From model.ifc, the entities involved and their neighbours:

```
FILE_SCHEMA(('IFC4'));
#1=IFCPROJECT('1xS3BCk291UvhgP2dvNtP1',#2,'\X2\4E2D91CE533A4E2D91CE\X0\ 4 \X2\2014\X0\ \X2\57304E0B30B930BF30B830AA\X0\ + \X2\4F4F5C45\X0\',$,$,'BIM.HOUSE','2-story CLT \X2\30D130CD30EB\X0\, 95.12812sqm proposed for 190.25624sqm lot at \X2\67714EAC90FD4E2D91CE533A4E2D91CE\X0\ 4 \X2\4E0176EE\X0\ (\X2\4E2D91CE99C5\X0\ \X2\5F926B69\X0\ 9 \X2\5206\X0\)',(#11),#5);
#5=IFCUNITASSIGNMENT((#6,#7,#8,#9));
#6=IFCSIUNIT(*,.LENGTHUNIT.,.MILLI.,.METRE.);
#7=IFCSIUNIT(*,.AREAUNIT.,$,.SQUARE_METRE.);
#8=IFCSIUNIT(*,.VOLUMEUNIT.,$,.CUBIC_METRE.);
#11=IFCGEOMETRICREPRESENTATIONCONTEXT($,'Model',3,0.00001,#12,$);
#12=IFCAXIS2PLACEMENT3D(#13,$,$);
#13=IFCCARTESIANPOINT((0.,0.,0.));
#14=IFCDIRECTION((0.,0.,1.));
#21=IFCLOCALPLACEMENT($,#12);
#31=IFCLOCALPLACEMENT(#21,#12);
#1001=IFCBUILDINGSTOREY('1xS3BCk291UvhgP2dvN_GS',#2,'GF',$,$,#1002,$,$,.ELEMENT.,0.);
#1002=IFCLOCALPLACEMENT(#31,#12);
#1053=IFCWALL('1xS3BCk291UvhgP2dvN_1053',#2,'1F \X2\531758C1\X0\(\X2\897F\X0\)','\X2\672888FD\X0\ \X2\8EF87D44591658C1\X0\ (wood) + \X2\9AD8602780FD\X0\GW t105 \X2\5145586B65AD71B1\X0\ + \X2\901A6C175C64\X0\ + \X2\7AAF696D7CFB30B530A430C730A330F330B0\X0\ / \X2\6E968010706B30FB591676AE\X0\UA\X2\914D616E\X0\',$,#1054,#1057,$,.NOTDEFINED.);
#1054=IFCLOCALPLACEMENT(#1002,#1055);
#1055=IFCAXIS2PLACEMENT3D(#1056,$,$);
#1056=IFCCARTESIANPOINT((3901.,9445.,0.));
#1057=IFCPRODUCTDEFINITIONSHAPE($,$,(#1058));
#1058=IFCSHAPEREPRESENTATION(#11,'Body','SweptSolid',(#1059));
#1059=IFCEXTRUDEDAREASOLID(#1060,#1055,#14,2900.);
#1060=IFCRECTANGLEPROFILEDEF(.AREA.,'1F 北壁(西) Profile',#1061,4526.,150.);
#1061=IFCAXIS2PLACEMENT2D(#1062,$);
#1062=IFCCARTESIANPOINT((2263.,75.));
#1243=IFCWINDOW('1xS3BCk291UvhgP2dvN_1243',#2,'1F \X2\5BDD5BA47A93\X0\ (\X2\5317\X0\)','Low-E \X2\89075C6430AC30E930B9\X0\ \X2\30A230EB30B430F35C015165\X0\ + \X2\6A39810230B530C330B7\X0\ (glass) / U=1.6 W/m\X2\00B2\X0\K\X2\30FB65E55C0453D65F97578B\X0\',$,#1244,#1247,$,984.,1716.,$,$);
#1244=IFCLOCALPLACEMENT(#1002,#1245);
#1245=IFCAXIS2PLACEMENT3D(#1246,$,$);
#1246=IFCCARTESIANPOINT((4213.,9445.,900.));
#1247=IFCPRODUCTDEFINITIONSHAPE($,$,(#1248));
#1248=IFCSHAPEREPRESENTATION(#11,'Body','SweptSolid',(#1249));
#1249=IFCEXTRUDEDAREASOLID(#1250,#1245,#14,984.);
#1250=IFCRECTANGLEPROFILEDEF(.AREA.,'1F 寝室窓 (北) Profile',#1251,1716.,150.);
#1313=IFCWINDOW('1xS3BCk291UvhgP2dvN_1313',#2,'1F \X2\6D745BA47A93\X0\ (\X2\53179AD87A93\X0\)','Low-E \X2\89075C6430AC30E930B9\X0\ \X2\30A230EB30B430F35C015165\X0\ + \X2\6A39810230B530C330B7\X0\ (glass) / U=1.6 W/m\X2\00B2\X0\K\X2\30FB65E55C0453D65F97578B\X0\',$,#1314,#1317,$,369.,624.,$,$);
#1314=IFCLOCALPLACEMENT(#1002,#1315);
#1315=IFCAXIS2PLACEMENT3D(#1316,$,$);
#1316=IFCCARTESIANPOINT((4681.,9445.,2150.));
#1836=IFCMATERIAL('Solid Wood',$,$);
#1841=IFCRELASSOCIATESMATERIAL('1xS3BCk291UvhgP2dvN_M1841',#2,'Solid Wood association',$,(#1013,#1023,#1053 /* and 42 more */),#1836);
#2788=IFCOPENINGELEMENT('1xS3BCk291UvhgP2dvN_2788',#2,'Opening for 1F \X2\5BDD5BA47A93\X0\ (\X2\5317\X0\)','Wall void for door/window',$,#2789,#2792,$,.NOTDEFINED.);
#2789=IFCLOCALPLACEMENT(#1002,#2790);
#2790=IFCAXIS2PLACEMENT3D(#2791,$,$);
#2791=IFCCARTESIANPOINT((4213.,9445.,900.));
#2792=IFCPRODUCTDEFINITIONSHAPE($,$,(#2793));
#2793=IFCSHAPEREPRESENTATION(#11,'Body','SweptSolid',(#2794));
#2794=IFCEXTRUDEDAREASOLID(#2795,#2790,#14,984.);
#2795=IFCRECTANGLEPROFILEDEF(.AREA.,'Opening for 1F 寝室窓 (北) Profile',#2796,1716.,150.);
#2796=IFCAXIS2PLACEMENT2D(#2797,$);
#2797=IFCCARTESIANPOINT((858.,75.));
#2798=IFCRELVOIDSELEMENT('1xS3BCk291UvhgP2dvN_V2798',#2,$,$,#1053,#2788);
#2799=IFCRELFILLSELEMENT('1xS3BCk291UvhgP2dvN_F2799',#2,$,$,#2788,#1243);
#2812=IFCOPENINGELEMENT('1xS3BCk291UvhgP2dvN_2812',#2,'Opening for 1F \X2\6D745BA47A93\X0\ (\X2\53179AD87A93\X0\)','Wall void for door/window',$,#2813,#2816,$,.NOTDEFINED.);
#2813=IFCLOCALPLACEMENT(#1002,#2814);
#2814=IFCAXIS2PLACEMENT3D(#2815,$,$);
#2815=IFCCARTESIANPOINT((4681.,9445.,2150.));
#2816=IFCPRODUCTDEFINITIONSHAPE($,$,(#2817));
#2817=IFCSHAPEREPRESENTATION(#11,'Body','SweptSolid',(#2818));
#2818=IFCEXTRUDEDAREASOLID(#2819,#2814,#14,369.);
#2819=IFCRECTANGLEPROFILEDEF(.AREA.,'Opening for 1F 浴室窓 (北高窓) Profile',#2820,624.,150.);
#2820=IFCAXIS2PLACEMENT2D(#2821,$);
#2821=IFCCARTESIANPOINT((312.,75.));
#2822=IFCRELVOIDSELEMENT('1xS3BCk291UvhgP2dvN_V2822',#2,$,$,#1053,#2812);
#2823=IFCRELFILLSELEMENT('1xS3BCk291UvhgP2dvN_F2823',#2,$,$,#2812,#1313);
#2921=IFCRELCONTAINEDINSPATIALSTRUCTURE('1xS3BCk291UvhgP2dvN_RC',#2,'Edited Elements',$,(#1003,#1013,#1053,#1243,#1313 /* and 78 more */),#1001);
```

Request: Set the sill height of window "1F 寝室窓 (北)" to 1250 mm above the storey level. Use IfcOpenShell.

```python
import numpy as np
import ifcopenshell
import ifcopenshell.api.geometry
import ifcopenshell.geom
import ifcopenshell.util.element
import ifcopenshell.util.placement
import ifcopenshell.util.shape
import ifcopenshell.util.unit

model = ifcopenshell.open("model.ifc")
unit_scale = ifcopenshell.util.unit.calculate_unit_scale(model)

window = model.by_guid("1xS3BCk291UvhgP2dvN_1243")
opening = window.FillsVoids[0].RelatingOpeningElement
storey = ifcopenshell.util.element.get_container(window, ifc_class="IfcBuildingStorey")
level = ifcopenshell.util.placement.get_local_placement(storey.ObjectPlacement)[2, 3]

# The opening's origin need not be at the sill, so measure its lowest point.
shape = ifcopenshell.geom.create_shape(ifcopenshell.geom.settings(), opening)
bottom = ifcopenshell.util.shape.get_shape_bottom_elevation(shape, shape.geometry) / unit_scale
dz = level + 1250.0 - bottom

shift = np.array([0.0, 0.0, dz])
# The window is not placed relative to its opening, so move both.
for product in (opening, window):
    matrix = ifcopenshell.util.placement.get_local_placement(product.ObjectPlacement)
    matrix[:3, 3] += shift
    ifcopenshell.api.geometry.edit_object_placement(model, product=product, matrix=matrix, is_si=False)

print(f"moved by {dz * unit_scale:+.3f} m")

model.write("model_edited.ifc")
```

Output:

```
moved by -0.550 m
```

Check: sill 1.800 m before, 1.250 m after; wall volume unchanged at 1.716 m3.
